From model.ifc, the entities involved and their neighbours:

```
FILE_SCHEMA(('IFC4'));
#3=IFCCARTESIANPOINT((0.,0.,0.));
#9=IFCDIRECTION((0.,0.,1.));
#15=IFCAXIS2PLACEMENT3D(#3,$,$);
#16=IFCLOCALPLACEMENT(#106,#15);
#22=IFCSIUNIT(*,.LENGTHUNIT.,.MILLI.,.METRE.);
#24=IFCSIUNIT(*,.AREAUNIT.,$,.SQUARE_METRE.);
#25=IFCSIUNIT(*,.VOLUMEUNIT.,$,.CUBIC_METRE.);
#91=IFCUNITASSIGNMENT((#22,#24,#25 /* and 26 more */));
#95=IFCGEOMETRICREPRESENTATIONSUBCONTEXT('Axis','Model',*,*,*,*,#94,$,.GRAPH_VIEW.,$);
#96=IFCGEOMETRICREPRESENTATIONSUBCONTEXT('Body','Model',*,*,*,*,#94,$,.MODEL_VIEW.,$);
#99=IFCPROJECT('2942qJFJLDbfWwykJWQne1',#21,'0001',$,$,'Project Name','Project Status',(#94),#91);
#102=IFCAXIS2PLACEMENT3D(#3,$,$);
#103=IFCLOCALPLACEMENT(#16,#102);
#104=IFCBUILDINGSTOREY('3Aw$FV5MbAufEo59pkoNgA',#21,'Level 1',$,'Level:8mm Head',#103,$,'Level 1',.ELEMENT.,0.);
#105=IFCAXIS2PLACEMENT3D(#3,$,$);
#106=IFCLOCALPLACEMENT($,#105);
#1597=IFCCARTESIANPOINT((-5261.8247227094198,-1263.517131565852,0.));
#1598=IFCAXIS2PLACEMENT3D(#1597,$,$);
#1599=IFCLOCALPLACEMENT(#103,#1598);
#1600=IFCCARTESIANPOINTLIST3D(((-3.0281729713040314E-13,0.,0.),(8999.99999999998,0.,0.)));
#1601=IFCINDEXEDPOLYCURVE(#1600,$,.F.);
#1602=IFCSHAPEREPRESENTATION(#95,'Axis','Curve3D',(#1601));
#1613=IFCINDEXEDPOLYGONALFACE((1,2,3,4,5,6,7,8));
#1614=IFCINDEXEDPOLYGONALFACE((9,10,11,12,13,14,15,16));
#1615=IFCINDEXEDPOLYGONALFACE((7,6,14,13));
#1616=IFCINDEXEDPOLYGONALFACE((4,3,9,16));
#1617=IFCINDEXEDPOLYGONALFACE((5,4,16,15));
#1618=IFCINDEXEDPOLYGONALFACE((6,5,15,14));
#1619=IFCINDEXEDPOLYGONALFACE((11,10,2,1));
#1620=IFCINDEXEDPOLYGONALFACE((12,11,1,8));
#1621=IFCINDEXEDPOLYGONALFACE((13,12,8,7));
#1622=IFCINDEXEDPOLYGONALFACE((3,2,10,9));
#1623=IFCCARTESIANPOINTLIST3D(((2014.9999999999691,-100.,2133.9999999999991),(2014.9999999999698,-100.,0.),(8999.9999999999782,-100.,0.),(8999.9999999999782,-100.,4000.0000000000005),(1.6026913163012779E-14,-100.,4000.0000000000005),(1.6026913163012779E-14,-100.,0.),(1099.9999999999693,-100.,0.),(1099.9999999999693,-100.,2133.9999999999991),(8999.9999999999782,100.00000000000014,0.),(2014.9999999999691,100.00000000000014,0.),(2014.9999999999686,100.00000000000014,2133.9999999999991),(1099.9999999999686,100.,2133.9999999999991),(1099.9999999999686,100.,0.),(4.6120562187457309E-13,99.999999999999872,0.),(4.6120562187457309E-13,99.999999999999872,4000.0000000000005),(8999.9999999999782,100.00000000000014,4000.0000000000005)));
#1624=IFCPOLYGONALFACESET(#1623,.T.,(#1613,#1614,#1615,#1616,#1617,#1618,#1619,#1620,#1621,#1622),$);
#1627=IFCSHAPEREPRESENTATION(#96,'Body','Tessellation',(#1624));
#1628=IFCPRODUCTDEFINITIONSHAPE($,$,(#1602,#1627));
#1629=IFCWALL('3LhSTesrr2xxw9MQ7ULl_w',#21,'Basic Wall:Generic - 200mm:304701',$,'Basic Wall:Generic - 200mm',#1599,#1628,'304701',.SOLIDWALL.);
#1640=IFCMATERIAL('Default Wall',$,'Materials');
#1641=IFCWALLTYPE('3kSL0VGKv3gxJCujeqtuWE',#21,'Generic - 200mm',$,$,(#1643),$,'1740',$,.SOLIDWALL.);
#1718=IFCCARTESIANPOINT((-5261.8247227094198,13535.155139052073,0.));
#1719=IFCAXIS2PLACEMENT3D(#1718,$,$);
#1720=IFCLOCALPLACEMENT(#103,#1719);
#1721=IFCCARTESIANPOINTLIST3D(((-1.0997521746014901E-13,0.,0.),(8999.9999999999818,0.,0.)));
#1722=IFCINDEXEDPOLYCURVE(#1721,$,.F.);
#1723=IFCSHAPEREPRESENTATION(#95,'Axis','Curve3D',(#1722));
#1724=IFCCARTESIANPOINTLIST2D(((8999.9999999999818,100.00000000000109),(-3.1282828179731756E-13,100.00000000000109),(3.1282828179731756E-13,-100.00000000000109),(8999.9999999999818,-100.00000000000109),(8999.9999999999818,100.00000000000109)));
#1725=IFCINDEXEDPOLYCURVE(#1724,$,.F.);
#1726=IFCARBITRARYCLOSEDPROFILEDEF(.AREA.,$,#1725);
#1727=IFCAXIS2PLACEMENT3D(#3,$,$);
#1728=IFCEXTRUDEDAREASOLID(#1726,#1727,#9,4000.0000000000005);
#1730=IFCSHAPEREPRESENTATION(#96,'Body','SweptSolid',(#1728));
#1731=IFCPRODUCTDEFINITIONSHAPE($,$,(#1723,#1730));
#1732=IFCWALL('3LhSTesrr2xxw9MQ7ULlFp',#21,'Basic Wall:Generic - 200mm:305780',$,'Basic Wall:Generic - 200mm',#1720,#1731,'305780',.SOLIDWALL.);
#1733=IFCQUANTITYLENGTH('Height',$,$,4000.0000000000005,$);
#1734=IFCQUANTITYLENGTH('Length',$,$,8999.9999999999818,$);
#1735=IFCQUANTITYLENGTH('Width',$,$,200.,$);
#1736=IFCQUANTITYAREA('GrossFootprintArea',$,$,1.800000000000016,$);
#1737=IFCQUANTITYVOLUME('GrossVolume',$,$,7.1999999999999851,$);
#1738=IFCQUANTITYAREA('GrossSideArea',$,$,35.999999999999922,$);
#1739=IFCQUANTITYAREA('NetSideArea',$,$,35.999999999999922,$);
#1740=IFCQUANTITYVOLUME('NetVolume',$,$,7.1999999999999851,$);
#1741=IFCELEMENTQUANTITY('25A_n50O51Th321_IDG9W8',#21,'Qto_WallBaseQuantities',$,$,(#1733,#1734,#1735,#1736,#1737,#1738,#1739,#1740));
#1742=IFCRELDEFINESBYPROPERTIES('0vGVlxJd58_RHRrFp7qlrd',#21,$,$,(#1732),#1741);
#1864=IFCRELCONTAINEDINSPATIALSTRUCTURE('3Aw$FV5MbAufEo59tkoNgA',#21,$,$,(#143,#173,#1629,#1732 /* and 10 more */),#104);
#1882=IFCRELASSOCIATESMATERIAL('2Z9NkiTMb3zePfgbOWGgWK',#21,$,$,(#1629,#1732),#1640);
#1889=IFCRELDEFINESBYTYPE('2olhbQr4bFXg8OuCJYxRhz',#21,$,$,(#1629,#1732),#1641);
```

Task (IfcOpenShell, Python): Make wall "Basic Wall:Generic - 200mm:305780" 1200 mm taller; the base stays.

```python
import ifcopenshell
import ifcopenshell.api.pset
import ifcopenshell.geom
import ifcopenshell.util.element
import ifcopenshell.util.representation
import ifcopenshell.util.shape
import ifcopenshell.util.unit

model = ifcopenshell.open("model.ifc")
unit_scale = ifcopenshell.util.unit.calculate_unit_scale(model)
area_scale = ifcopenshell.util.unit.calculate_unit_scale(model, "AREAUNIT")
volume_scale = ifcopenshell.util.unit.calculate_unit_scale(model, "VOLUMEUNIT")
settings = ifcopenshell.geom.settings()


def volume(element):
    """Net volume in cubic metres, openings subtracted."""
    shape = ifcopenshell.geom.create_shape(settings, element)
    return ifcopenshell.util.shape.get_volume(shape.geometry)


wall = model.by_guid("3LhSTesrr2xxw9MQ7ULlFp")
before = volume(wall)

body = ifcopenshell.util.representation.get_representation(wall, "Model", "Body")
solid = body.Items[0]
old_height = solid.Depth
solid.Depth += 1.2 / unit_scale
after = volume(wall)
thickness = 0.2  # wall thickness in metres

# Update the stored height, areas and volumes.
qto = model.by_id(ifcopenshell.util.element.get_pset(wall, "Qto_WallBaseQuantities", should_inherit=False)["id"])
ifcopenshell.api.pset.edit_qto(model, qto=qto, properties={
    "Height": solid.Depth,
    "GrossVolume": ifcopenshell.util.element.get_pset(wall, "Qto_WallBaseQuantities", "GrossVolume") * solid.Depth / old_height,
    "GrossSideArea": ifcopenshell.util.element.get_pset(wall, "Qto_WallBaseQuantities", "GrossSideArea") * solid.Depth / old_height,
    "NetSideArea": after / thickness / area_scale,
    "NetVolume": after / volume_scale,
})

print(f"height {old_height:g} -> {solid.Depth:g}, volume {before:.3f} -> {after:.3f} m3")

model.write("model_rev.ifc")
```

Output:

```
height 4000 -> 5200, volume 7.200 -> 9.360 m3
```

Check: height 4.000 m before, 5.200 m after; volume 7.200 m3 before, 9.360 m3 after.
